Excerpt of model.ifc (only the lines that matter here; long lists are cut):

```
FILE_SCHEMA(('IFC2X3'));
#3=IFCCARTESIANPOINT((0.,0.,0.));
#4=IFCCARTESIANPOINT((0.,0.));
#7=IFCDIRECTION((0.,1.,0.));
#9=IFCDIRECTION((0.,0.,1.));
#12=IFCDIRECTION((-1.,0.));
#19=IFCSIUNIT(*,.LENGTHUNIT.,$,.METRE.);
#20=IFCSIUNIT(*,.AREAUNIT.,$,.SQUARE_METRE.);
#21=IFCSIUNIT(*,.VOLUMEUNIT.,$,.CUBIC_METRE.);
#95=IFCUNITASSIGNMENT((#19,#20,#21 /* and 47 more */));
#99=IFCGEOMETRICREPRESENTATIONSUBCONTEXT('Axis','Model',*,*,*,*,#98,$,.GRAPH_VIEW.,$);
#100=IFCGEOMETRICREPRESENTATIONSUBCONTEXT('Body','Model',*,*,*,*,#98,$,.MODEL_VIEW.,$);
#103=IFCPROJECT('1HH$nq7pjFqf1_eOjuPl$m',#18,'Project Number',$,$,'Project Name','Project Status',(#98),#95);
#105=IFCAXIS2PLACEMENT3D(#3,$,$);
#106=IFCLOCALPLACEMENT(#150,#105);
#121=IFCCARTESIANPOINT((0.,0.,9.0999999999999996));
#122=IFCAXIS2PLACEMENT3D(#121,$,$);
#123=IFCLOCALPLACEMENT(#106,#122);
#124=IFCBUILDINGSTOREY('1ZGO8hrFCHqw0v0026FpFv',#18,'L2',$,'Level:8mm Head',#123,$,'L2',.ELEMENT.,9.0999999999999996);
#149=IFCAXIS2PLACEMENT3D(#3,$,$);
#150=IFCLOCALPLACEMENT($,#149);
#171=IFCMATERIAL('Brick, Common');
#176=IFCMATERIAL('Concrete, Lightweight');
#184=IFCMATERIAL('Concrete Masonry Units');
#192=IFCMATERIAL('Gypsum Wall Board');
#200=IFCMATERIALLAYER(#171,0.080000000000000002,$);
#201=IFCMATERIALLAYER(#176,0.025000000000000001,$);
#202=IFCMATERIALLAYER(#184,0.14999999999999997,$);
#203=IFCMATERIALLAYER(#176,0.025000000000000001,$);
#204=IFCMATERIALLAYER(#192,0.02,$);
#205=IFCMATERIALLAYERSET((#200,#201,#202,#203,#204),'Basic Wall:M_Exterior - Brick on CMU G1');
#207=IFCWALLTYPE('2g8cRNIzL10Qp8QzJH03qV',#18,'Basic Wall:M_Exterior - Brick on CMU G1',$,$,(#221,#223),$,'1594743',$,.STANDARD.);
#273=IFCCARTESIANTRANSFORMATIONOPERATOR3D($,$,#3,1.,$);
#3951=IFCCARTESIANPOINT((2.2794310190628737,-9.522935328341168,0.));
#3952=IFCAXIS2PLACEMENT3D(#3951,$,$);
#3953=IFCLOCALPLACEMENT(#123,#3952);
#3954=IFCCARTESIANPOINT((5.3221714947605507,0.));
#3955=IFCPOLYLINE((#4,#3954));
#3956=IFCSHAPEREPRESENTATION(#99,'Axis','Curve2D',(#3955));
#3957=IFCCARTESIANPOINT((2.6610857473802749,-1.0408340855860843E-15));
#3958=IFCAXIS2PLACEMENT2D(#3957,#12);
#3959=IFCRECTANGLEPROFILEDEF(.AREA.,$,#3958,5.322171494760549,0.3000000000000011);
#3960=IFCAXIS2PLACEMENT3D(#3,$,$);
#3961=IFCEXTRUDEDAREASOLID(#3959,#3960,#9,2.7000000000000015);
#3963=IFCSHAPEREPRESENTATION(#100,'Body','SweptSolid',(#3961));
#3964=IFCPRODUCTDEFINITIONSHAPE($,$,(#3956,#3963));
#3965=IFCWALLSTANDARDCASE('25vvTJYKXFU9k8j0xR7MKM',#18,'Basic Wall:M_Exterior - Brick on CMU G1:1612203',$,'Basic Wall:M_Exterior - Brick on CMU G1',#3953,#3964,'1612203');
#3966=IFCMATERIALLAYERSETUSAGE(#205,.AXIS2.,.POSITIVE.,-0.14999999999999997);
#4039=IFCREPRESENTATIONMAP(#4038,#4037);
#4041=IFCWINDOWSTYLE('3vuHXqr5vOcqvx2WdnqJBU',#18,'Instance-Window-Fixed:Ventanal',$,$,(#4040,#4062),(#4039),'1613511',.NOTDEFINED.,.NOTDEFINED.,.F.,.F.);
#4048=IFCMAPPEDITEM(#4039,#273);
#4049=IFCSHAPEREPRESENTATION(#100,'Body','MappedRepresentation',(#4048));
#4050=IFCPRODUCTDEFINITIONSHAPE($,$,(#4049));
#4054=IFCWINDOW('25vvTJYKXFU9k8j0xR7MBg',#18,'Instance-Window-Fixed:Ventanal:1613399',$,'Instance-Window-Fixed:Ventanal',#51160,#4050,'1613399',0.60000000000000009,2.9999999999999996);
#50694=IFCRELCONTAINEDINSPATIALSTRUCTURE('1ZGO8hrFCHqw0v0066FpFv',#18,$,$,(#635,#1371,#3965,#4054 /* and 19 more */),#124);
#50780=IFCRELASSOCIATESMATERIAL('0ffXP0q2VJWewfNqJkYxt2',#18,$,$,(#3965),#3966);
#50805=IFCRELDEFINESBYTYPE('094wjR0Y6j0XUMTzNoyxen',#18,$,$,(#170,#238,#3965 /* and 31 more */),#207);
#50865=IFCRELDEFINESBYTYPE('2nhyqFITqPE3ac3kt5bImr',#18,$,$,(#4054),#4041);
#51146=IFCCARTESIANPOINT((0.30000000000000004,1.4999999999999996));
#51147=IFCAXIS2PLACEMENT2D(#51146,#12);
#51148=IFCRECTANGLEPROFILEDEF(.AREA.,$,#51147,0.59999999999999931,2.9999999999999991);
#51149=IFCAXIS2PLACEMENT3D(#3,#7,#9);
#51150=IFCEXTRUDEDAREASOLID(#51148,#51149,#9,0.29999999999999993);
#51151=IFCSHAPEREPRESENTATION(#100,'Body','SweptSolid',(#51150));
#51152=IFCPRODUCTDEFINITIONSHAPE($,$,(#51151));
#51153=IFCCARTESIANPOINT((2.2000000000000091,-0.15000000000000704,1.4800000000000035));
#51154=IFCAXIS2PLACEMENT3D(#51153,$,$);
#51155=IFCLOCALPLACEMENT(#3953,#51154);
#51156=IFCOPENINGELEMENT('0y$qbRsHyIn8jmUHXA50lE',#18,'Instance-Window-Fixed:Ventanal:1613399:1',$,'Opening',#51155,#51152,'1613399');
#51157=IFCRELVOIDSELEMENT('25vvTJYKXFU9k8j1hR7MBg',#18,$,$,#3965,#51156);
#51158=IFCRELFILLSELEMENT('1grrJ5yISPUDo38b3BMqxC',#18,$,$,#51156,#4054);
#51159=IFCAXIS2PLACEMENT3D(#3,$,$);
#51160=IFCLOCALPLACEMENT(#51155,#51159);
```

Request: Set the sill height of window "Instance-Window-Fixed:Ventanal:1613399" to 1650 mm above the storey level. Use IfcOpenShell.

```python
import numpy as np
import ifcopenshell
import ifcopenshell.api.geometry
import ifcopenshell.geom
import ifcopenshell.util.element
import ifcopenshell.util.placement
import ifcopenshell.util.shape
import ifcopenshell.util.unit

model = ifcopenshell.open("model.ifc")
unit_scale = ifcopenshell.util.unit.calculate_unit_scale(model)

window = model.by_id(4054)
opening = window.FillsVoids[0].RelatingOpeningElement
storey = ifcopenshell.util.element.get_container(window, ifc_class="IfcBuildingStorey")
level = ifcopenshell.util.placement.get_local_placement(storey.ObjectPlacement)[2, 3]

# The opening's origin need not be at the sill, so measure its lowest point.
shape = ifcopenshell.geom.create_shape(ifcopenshell.geom.settings(), opening)
bottom = ifcopenshell.util.shape.get_shape_bottom_elevation(shape, shape.geometry) / unit_scale
dz = level + 1.65 / unit_scale - bottom

shift = np.array([0.0, 0.0, dz])
# The window is placed relative to its opening, so it follows when the opening moves.
matrix = ifcopenshell.util.placement.get_local_placement(opening.ObjectPlacement)
matrix[:3, 3] += shift
ifcopenshell.api.geometry.edit_object_placement(
    model, product=opening, matrix=matrix, is_si=False, should_transform_children=True
)

print(f"moved by {dz * unit_scale:+.3f} m")

model.write("model_edited.ifc")
```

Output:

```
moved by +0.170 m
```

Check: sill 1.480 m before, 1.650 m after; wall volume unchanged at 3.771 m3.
